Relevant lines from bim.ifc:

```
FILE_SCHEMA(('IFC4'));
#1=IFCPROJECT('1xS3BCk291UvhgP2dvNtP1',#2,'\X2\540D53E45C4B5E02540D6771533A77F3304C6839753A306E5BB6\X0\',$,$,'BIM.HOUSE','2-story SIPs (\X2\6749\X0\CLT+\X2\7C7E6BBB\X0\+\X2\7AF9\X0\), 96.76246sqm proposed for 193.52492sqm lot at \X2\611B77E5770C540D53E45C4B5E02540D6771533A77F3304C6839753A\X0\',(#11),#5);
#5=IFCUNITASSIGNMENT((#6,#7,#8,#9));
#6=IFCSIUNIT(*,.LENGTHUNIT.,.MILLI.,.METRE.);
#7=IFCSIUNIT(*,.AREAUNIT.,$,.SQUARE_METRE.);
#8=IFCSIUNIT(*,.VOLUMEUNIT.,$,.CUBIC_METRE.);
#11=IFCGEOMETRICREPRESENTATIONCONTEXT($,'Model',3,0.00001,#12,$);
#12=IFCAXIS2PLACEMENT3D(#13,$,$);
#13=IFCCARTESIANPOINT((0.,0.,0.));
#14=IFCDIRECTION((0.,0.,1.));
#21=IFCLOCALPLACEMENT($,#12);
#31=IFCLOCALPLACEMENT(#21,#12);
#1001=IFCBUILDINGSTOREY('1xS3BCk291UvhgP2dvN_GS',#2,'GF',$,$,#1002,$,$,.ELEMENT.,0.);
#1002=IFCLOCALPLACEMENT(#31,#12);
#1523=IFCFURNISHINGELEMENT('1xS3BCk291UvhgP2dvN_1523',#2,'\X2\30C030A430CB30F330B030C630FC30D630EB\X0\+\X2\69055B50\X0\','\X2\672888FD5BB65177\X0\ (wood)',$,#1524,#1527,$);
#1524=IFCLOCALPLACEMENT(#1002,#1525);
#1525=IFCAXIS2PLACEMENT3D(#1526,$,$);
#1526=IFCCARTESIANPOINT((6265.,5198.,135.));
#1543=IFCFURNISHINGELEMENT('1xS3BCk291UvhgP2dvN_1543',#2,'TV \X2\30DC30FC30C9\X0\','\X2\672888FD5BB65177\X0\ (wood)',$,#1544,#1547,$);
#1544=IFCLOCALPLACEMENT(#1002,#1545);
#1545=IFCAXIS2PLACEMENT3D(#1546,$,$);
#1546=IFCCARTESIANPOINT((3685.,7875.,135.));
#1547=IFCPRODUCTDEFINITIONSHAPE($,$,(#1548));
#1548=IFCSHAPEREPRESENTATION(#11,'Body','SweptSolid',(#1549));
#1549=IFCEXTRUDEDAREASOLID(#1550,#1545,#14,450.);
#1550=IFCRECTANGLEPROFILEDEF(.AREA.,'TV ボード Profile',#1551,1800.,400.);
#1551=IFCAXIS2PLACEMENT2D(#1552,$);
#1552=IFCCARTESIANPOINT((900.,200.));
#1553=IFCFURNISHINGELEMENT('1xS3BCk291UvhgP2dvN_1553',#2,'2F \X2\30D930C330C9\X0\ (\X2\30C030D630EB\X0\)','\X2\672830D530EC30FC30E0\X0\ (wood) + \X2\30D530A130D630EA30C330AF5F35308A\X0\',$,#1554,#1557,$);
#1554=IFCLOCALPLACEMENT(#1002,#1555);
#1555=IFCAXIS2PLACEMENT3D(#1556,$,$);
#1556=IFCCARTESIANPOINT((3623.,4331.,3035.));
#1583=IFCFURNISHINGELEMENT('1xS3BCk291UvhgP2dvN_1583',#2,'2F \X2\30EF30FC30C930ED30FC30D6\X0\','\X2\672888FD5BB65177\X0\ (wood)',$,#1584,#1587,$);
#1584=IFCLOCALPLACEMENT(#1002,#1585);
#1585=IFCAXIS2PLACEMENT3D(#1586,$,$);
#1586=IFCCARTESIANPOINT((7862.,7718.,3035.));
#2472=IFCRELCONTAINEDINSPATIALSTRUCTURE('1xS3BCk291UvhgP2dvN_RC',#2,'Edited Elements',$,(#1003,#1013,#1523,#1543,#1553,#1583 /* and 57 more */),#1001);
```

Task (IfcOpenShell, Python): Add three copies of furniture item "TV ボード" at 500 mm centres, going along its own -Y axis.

```python
import ifcopenshell
import ifcopenshell.api.geometry
import ifcopenshell.api.root
import ifcopenshell.util.element
import ifcopenshell.util.placement

model = ifcopenshell.open("bim.ifc")


def reuse_history(source, copy):
    """copy_class also copies each property set's owner history, people and application; keep the originals."""
    for rel in copy.IsDefinedBy:
        if rel.is_a("IfcRelDefinesByProperties") and (history := rel.RelatingPropertyDefinition.OwnerHistory):
            rel.RelatingPropertyDefinition.OwnerHistory = source.OwnerHistory
            ifcopenshell.util.element.remove_deep2(model, history)


source = model.by_guid("1xS3BCk291UvhgP2dvN_1543")
base = ifcopenshell.util.placement.get_local_placement(source.ObjectPlacement)
step = -base[:3, 1] * 500.0

for i in range(1, 4):
    copy = ifcopenshell.api.root.copy_class(model, product=source)
    copy.Representation = ifcopenshell.util.element.copy_deep(
        model, source.Representation, exclude=["IfcGeometricRepresentationContext", "IfcRepresentationMap"]
    )
    reuse_history(source, copy)
    matrix = base.copy()
    matrix[:3, 3] += i * step
    print("added at", matrix[:3, 3].round(3) + 0.0)
    ifcopenshell.api.geometry.edit_object_placement(model, product=copy, matrix=matrix, is_si=False)

model.write("bim_edited.ifc")
```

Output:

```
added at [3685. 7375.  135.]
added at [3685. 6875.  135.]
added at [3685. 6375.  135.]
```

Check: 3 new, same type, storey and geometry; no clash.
